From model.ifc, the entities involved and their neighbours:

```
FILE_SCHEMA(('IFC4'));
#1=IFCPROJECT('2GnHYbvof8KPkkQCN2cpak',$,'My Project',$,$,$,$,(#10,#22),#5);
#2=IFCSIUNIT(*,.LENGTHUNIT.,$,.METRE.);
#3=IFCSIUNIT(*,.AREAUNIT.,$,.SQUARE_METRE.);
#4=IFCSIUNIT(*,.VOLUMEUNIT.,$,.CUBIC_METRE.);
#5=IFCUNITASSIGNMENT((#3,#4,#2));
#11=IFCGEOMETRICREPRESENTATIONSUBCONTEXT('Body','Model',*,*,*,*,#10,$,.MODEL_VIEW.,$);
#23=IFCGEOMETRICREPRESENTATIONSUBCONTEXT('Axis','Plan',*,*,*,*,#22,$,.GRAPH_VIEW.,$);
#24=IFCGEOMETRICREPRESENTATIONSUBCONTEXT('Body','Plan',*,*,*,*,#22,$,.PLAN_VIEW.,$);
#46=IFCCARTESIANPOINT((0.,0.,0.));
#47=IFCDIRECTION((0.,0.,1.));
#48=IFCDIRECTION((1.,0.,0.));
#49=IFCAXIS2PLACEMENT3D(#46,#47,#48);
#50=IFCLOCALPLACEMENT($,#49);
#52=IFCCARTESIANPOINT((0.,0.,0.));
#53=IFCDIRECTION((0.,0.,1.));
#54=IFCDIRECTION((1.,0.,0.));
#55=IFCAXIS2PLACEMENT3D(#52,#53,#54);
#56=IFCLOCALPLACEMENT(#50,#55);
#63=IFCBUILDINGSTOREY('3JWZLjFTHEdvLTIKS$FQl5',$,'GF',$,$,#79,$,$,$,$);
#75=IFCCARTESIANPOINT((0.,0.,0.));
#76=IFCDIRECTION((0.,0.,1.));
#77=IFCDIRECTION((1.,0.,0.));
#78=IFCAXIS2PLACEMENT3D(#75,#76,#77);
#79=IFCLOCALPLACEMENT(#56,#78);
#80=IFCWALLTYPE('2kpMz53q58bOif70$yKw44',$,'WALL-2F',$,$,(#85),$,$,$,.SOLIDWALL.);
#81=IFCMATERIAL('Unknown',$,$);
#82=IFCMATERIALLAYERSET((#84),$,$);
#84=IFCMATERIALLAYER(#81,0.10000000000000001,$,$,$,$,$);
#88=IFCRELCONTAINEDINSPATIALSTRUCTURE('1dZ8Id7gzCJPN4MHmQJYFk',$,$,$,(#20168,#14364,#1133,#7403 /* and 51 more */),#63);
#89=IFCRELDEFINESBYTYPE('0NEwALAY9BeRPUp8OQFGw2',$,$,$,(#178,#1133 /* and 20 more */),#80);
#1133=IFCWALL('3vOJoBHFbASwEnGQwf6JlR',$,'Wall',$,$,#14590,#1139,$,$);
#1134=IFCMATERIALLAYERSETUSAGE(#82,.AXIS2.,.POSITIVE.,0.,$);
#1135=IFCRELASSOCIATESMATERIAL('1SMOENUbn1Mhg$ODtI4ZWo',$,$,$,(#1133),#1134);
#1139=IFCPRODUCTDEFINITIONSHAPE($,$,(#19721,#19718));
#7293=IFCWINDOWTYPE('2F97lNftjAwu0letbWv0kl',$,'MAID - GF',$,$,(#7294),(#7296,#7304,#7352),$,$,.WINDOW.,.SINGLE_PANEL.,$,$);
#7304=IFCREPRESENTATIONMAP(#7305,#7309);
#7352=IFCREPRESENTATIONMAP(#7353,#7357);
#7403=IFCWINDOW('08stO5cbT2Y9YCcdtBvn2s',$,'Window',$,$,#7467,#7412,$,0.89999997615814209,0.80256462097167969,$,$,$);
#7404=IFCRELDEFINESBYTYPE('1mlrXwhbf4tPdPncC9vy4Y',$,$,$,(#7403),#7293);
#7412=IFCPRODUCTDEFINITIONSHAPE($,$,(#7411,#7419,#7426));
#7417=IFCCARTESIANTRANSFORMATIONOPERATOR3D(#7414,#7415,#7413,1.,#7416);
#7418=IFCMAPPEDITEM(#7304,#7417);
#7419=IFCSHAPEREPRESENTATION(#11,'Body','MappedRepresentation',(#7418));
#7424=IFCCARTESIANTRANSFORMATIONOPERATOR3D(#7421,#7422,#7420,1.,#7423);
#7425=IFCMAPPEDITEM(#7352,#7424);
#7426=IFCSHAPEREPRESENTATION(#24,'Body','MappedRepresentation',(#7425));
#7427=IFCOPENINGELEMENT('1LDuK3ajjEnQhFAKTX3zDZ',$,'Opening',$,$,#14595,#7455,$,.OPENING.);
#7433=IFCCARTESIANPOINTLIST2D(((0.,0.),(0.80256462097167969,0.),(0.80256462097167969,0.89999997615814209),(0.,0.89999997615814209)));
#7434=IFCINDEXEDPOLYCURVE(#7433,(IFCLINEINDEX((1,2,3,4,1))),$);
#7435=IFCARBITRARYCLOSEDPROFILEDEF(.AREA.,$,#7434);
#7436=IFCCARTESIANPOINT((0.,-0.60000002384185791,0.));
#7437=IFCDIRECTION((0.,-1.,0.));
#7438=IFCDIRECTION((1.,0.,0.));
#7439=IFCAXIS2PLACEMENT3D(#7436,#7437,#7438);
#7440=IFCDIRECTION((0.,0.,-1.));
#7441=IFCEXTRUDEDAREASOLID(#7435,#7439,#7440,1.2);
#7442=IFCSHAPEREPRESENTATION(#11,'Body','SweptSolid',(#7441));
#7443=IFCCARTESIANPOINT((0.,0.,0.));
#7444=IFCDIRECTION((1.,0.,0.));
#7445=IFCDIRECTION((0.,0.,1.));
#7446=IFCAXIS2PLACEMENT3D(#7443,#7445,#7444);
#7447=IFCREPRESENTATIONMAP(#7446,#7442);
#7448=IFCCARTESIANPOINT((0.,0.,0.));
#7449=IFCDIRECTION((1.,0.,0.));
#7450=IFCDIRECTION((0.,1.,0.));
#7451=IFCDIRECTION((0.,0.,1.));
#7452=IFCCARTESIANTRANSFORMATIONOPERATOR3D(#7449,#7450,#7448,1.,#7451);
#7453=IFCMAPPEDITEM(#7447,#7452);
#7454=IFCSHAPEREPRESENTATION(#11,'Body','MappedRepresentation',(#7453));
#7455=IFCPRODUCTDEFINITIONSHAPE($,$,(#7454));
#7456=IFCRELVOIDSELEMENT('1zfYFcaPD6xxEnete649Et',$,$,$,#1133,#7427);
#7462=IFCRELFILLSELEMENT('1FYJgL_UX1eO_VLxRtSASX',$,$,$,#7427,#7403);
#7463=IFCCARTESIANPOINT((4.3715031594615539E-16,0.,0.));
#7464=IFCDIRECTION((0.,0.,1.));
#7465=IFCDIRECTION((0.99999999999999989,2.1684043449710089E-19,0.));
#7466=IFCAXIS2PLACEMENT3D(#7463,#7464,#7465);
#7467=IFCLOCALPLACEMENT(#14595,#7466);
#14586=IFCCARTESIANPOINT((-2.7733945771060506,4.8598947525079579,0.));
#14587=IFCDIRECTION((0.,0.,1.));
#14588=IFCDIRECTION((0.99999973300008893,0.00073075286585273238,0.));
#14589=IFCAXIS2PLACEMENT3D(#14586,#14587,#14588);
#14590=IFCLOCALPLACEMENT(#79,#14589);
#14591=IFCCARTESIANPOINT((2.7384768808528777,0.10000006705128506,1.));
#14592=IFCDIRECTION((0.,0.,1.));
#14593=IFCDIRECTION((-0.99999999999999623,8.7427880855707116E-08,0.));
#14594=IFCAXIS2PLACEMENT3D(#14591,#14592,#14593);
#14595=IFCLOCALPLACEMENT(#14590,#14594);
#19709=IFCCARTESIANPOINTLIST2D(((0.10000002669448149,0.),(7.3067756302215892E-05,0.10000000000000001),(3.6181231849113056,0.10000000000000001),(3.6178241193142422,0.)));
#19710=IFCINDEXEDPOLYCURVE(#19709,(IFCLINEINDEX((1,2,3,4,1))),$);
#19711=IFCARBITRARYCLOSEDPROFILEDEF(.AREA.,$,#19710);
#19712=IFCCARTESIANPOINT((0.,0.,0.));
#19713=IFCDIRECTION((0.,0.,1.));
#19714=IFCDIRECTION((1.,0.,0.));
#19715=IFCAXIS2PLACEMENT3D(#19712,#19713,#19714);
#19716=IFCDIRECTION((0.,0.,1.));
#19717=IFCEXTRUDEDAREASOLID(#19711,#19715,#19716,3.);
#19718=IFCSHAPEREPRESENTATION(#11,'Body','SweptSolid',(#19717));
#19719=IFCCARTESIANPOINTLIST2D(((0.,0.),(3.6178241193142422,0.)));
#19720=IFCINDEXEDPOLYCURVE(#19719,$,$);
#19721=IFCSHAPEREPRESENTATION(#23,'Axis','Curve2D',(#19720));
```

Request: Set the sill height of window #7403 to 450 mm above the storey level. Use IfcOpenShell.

```python
import numpy as np
import ifcopenshell
import ifcopenshell.api.geometry
import ifcopenshell.geom
import ifcopenshell.util.element
import ifcopenshell.util.placement
import ifcopenshell.util.shape
import ifcopenshell.util.unit

model = ifcopenshell.open("model.ifc")
unit_scale = ifcopenshell.util.unit.calculate_unit_scale(model)

window = model.by_guid("08stO5cbT2Y9YCcdtBvn2s")
opening = window.FillsVoids[0].RelatingOpeningElement
storey = ifcopenshell.util.element.get_container(window, ifc_class="IfcBuildingStorey")
level = ifcopenshell.util.placement.get_local_placement(storey.ObjectPlacement)[2, 3]

# The opening's origin need not be at the sill, so measure its lowest point.
shape = ifcopenshell.geom.create_shape(ifcopenshell.geom.settings(), opening)
bottom = ifcopenshell.util.shape.get_shape_bottom_elevation(shape, shape.geometry) / unit_scale
dz = level + 0.45 - bottom

shift = np.array([0.0, 0.0, dz])
# The window is placed relative to its opening, so it follows when the opening moves.
matrix = ifcopenshell.util.placement.get_local_placement(opening.ObjectPlacement)
matrix[:3, 3] += shift
ifcopenshell.api.geometry.edit_object_placement(
    model, product=opening, matrix=matrix, is_si=False, should_transform_children=True
)

print(f"moved by {dz * unit_scale:+.3f} m")

model.write("model_rev.ifc")
```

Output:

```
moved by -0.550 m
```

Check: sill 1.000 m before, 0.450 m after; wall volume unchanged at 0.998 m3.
